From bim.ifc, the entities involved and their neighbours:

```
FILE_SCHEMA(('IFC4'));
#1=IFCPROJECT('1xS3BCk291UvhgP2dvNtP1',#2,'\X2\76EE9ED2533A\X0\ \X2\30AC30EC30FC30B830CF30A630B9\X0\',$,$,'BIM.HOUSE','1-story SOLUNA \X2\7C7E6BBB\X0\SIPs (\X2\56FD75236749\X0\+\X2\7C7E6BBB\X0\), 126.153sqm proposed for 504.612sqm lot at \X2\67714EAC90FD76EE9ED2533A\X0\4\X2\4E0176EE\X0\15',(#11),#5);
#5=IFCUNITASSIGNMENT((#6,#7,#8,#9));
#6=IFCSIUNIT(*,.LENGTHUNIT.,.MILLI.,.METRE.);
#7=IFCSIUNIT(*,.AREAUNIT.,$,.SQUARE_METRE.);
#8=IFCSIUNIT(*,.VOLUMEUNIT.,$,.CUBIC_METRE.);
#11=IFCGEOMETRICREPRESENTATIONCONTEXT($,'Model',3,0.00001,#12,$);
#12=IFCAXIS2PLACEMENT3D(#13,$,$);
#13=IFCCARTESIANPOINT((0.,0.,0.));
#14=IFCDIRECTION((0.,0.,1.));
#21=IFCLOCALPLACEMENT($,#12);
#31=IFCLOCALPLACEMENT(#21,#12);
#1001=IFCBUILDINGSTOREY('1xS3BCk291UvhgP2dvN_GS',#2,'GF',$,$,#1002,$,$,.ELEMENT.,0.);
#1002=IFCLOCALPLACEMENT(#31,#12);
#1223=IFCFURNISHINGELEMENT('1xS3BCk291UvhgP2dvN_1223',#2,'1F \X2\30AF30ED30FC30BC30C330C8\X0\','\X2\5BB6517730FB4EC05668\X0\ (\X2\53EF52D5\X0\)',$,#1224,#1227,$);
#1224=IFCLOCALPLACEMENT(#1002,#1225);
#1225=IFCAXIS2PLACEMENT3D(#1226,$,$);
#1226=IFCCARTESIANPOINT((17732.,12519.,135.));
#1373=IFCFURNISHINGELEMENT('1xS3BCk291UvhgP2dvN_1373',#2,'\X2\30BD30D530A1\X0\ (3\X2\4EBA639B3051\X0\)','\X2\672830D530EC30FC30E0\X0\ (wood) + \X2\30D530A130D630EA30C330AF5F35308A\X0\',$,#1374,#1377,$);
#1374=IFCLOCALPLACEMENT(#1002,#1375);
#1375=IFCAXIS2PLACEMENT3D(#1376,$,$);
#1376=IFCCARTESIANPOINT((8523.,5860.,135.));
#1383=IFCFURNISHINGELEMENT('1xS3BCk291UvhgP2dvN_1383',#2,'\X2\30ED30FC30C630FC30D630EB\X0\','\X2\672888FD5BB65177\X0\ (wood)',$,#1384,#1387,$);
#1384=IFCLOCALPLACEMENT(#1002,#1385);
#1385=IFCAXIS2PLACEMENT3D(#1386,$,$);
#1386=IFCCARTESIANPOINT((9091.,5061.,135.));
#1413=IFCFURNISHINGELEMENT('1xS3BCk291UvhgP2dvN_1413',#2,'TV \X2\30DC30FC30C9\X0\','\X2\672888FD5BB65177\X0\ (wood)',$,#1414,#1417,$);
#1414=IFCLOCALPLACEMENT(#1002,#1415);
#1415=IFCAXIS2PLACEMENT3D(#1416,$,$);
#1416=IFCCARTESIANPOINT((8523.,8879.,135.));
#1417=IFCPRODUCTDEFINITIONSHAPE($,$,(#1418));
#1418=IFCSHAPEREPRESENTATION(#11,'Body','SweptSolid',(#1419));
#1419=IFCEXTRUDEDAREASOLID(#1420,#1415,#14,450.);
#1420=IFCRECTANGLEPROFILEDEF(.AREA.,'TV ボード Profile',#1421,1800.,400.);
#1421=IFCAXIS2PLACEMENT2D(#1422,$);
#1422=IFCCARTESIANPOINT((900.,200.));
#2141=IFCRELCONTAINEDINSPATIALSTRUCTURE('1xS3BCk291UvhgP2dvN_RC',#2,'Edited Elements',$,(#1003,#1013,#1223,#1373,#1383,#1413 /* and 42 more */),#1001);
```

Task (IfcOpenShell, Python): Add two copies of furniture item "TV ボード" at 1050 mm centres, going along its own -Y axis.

```python
import ifcopenshell
import ifcopenshell.api.geometry
import ifcopenshell.api.root
import ifcopenshell.util.element
import ifcopenshell.util.placement
import ifcopenshell.util.unit

model = ifcopenshell.open("bim.ifc")
unit_scale = ifcopenshell.util.unit.calculate_unit_scale(model)


def reuse_history(source, copy):
    """copy_class also copies each property set's owner history, people and application; keep the originals."""
    for rel in copy.IsDefinedBy:
        if rel.is_a("IfcRelDefinesByProperties") and (history := rel.RelatingPropertyDefinition.OwnerHistory):
            rel.RelatingPropertyDefinition.OwnerHistory = source.OwnerHistory
            ifcopenshell.util.element.remove_deep2(model, history)


source = model.by_guid("1xS3BCk291UvhgP2dvN_1413")
base = ifcopenshell.util.placement.get_local_placement(source.ObjectPlacement)
step = -base[:3, 1] * 1.05 / unit_scale

for i in range(1, 3):
    copy = ifcopenshell.api.root.copy_class(model, product=source)
    copy.Representation = ifcopenshell.util.element.copy_deep(
        model, source.Representation, exclude=["IfcGeometricRepresentationContext", "IfcRepresentationMap"]
    )
    reuse_history(source, copy)
    matrix = base.copy()
    matrix[:3, 3] += i * step
    print("added at", matrix[:3, 3].round(3) + 0.0)
    ifcopenshell.api.geometry.edit_object_placement(model, product=copy, matrix=matrix, is_si=False)

model.write("bim_edited.ifc")
```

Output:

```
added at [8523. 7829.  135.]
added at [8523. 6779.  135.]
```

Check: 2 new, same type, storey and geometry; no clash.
